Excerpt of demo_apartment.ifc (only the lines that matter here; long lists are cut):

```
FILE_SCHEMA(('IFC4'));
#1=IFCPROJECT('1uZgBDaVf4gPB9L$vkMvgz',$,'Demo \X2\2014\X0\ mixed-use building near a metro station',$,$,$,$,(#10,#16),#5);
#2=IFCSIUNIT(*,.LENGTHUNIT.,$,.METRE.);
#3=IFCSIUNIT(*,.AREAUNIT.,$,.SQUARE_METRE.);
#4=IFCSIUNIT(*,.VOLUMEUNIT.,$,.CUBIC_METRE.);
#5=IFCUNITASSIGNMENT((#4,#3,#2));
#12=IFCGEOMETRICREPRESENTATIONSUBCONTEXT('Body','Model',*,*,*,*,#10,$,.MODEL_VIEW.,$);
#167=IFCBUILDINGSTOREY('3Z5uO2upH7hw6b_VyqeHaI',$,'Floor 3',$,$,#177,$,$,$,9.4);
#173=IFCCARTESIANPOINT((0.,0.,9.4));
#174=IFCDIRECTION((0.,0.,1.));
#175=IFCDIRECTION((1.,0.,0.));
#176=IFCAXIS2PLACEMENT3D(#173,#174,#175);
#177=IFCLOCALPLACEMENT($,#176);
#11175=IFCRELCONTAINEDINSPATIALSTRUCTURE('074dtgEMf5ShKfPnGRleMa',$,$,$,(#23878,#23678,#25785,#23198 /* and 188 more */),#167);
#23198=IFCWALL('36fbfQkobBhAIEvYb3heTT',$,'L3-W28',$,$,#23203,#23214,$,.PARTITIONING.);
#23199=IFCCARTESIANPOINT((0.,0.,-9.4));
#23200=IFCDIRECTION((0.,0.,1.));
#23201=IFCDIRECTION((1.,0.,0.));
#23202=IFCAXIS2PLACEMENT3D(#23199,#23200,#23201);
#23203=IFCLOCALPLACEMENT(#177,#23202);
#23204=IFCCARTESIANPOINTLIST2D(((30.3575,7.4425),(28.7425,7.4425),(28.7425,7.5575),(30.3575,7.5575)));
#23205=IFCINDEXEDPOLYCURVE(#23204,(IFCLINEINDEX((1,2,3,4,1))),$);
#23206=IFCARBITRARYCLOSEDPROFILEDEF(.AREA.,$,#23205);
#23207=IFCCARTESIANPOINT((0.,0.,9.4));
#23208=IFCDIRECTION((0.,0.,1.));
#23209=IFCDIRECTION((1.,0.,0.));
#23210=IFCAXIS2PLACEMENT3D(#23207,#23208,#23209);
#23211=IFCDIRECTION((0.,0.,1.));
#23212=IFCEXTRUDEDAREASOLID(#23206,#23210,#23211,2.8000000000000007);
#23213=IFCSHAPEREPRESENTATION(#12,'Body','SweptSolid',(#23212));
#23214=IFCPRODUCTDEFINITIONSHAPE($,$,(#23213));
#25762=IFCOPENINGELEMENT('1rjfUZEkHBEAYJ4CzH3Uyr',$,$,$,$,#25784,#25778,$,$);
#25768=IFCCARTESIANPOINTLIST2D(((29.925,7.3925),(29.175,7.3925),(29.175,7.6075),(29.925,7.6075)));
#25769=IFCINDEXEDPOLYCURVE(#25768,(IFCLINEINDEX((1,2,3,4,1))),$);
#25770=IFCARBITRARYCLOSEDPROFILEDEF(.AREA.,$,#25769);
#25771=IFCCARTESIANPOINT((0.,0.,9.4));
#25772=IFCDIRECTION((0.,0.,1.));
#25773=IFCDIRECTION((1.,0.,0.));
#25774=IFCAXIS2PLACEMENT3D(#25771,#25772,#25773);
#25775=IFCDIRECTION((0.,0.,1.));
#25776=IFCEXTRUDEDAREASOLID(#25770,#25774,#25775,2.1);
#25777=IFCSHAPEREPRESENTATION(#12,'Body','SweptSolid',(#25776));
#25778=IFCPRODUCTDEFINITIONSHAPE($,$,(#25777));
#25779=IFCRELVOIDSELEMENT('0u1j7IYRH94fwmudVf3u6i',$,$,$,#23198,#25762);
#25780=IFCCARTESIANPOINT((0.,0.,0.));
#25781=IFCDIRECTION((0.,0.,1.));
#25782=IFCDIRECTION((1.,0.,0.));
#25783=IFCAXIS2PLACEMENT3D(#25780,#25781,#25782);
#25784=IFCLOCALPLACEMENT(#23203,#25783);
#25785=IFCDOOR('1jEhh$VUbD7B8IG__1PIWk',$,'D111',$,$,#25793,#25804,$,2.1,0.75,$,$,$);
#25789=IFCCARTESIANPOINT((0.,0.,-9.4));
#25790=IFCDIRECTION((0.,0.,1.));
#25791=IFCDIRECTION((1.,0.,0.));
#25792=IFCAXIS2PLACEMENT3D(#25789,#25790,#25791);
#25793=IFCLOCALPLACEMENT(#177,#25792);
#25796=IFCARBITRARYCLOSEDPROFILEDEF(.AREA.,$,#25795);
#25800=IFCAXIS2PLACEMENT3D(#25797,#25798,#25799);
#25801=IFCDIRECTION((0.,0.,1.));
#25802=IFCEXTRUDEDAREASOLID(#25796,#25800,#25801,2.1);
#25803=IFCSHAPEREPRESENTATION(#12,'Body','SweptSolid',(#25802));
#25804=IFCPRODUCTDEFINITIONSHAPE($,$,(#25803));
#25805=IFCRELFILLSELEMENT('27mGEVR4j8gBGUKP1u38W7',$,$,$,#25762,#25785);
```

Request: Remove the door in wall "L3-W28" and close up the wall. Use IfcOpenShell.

```python
import ifcopenshell
import ifcopenshell.api.feature
import ifcopenshell.api.root
import ifcopenshell.geom
import ifcopenshell.util.shape

model = ifcopenshell.open("demo_apartment.ifc")
settings = ifcopenshell.geom.settings()


def volume(element):
    """Net volume in cubic metres, openings subtracted."""
    shape = ifcopenshell.geom.create_shape(settings, element)
    return ifcopenshell.util.shape.get_volume(shape.geometry)


door = model.by_guid("1jEhh$VUbD7B8IG__1PIWk")
opening = door.FillsVoids[0].RelatingOpeningElement
wall = opening.VoidsElements[0].RelatingBuildingElement
before = volume(wall)

ifcopenshell.api.root.remove_product(model, product=door)
ifcopenshell.api.feature.remove_feature(model, feature=opening)

after = volume(wall)

print(f"wall volume {before:.3f} -> {after:.3f} m3")

model.write("demo_apartment_v2.ifc")
```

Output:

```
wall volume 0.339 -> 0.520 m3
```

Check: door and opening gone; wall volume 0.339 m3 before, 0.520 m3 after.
